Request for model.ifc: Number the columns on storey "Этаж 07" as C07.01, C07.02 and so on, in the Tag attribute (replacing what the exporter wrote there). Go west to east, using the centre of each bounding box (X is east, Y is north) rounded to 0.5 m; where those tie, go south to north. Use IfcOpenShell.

First a look at what the model holds.

```python
import ifcopenshell
import ifcopenshell.util.element
import ifcopenshell.util.placement

model = ifcopenshell.open("model.ifc")
print(model.schema)
storey = next(s for s in model.by_type("IfcBuildingStorey") if s.Name == "Этаж 07")
columns = [e for e in ifcopenshell.util.element.get_decomposition(storey) if e.is_a("IfcColumn")]
for e in sorted(columns, key=lambda e: e.id()):
    origin = ifcopenshell.util.placement.get_local_placement(e.ObjectPlacement)[:3, 3]
    print(e.id(), e.Tag, e.Name, origin.round(2) + 0.0, sep=" | ")
```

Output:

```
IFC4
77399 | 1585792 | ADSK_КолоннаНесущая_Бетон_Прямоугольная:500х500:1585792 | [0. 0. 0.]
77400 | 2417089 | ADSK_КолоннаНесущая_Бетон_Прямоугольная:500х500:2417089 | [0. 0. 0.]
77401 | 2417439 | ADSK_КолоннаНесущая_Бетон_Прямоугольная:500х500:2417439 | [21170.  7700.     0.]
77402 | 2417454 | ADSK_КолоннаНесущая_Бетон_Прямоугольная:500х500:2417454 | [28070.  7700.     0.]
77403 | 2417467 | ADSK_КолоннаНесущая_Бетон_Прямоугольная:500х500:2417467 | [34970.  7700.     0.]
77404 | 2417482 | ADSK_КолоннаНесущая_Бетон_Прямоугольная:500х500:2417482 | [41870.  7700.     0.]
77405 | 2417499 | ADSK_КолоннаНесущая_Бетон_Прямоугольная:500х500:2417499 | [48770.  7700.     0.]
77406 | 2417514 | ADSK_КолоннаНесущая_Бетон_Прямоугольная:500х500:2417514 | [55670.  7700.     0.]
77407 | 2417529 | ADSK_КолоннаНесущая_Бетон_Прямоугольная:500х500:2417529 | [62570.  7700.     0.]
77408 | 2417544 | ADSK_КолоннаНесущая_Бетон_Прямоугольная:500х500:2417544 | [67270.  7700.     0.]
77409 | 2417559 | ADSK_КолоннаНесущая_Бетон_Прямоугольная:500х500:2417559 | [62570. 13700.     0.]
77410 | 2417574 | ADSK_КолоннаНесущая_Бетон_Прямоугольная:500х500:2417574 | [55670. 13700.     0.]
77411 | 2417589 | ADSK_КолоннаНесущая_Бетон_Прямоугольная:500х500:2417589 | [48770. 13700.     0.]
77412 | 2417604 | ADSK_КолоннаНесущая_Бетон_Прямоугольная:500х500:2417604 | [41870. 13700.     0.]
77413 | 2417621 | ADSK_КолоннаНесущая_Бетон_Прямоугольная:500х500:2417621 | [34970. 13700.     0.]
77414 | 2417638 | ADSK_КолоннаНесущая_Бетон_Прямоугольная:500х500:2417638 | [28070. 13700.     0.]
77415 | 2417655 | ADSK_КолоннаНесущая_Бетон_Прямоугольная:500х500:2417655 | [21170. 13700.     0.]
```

```python
import ifcopenshell
import ifcopenshell.geom
import ifcopenshell.util.element
import ifcopenshell.util.shape

model = ifcopenshell.open("model.ifc")
settings = ifcopenshell.geom.settings()
settings.set("use-world-coords", True)


def centre(element):
    shape = ifcopenshell.geom.create_shape(settings, element)
    return ifcopenshell.util.shape.get_bbox_centroid(shape.geometry)


storey = next(s for s in model.by_type("IfcBuildingStorey") if s.Name == "Этаж 07")
columns = [e for e in ifcopenshell.util.element.get_decomposition(storey) if e.is_a("IfcColumn")]

# Insertion points can sit at a corner or the storey origin, so sort by the geometry (in metres).
centres = {e: centre(e) for e in columns}
columns.sort(key=lambda e: (round(centres[e][0] / 0.5), centres[e][1]))

for i, e in enumerate(columns, start=1):
    number = f"C07.{i:02d}"
    e.Tag = number
    print(e.id(), number)

model.write("model-out.ifc")
```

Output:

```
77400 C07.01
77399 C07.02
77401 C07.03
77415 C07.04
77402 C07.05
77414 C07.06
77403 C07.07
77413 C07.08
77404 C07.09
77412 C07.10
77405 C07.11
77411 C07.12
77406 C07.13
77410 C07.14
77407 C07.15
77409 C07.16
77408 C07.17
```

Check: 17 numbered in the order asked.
